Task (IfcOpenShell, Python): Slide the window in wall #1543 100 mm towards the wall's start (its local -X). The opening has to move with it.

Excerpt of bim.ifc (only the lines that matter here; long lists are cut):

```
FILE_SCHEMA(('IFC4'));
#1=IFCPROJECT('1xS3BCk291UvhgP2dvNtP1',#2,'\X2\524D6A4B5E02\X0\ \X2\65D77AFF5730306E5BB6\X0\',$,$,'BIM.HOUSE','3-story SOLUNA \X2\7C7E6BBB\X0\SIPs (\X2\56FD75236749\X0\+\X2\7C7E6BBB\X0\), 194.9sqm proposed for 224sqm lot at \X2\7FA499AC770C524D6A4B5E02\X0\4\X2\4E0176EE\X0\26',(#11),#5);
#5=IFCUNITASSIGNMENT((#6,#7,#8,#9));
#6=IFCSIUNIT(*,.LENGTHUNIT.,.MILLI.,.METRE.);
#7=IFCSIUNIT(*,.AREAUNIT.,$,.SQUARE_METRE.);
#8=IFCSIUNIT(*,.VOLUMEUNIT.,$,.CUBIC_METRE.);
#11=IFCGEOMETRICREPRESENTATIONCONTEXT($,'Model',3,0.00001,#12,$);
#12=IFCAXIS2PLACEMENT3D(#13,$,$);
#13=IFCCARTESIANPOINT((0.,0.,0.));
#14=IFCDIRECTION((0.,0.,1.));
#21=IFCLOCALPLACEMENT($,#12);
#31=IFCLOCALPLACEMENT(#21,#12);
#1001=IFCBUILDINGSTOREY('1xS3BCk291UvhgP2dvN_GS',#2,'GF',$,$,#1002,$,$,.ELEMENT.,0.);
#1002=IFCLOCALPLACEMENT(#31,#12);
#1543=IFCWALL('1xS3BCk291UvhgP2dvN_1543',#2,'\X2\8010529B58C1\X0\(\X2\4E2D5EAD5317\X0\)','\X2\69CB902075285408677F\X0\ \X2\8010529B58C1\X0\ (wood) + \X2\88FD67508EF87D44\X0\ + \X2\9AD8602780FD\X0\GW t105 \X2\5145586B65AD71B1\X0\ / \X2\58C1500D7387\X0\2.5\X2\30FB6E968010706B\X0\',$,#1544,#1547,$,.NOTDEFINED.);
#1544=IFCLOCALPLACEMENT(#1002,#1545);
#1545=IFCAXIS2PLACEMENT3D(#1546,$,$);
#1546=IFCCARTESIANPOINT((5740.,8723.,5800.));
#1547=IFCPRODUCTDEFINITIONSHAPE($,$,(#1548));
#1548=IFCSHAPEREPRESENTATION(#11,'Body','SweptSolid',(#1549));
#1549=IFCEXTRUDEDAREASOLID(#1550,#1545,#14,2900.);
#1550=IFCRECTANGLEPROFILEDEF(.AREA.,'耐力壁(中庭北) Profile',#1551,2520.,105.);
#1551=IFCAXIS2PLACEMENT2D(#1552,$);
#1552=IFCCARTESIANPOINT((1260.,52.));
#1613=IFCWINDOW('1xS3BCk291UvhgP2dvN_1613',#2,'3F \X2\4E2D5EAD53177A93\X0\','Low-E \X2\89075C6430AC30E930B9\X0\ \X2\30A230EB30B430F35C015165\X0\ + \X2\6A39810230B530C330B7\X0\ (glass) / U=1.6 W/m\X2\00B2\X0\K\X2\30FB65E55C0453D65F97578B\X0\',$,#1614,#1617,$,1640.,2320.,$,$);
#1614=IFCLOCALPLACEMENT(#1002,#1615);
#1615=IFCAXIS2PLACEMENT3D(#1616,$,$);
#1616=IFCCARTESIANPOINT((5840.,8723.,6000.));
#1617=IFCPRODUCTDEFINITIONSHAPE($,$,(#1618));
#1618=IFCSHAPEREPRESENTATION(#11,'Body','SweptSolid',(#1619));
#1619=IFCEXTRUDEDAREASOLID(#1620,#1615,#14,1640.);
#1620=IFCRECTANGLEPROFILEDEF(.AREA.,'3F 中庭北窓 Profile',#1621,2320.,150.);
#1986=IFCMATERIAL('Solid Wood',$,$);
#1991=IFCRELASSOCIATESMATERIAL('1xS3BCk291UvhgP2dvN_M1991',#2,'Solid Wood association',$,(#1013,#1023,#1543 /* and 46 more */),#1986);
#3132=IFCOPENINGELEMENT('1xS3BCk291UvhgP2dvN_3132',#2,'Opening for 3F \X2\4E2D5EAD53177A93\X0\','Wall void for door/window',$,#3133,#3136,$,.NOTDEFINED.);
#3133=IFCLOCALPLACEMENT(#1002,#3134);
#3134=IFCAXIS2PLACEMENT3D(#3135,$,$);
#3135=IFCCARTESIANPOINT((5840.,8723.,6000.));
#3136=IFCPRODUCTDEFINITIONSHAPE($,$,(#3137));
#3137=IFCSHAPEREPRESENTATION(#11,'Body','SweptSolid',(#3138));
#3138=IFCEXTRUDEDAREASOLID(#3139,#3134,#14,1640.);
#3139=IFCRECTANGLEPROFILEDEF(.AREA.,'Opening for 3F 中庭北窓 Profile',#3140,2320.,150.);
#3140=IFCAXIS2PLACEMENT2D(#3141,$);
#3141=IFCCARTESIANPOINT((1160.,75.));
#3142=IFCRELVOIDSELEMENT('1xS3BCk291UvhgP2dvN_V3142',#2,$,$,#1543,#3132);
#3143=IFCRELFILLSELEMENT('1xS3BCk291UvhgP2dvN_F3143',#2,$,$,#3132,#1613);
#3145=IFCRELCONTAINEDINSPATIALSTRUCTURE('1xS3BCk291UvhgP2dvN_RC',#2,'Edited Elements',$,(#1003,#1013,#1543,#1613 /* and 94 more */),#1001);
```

```python
import ifcopenshell
import ifcopenshell.api.geometry
import ifcopenshell.util.placement
import ifcopenshell.util.unit

model = ifcopenshell.open("bim.ifc")
unit_scale = ifcopenshell.util.unit.calculate_unit_scale(model)

window = model.by_guid("1xS3BCk291UvhgP2dvN_1613")
opening = window.FillsVoids[0].RelatingOpeningElement
wall = opening.VoidsElements[0].RelatingBuildingElement

wall_matrix = ifcopenshell.util.placement.get_local_placement(wall.ObjectPlacement)
shift = wall_matrix[:3, 0] * -0.1 / unit_scale
before = ifcopenshell.util.placement.get_local_placement(window.ObjectPlacement)[:3, 3].copy()

# The window is not placed relative to its opening, so move both.
for product in (opening, window):
    matrix = ifcopenshell.util.placement.get_local_placement(product.ObjectPlacement)
    matrix[:3, 3] += shift
    ifcopenshell.api.geometry.edit_object_placement(model, product=product, matrix=matrix, is_si=False)

after = ifcopenshell.util.placement.get_local_placement(window.ObjectPlacement)[:3, 3]
print("window moved by", (after - before).round(3) + 0.0)

model.write("bim_updated.ifc")
```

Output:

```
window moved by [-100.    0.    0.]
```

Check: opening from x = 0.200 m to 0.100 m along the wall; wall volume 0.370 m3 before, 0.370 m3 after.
